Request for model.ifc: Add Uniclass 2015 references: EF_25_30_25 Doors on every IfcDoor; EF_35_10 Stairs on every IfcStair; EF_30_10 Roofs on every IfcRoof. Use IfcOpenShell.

First a look at what the model holds.

```python
import ifcopenshell

model = ifcopenshell.open("model.ifc")
print(model.schema)
print("classifications:", [c.Name for c in model.by_type("IfcClassification")])
for ifc_class in ("IfcDoor", "IfcRoof", "IfcStair", "IfcWall", "IfcWindow"):
    print(ifc_class, len(model.by_type(ifc_class)))
```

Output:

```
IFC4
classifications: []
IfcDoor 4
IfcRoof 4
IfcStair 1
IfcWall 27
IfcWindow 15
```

```python
import ifcopenshell
import ifcopenshell.api.classification

model = ifcopenshell.open("model.ifc")

system = ifcopenshell.api.classification.add_classification(model, classification="Uniclass 2015")

codes = {
    "IfcDoor": ("EF_25_30_25", "Doors"),
    "IfcStair": ("EF_35_10", "Stairs"),
    "IfcRoof": ("EF_30_10", "Roofs"),
}
for ifc_class, (code, name) in codes.items():
    products = model.by_type(ifc_class)
    ifcopenshell.api.classification.add_reference(
        model, products=products, classification=system, identification=code, name=name
    )
    print(code, len(products))

model.write("model_v2.ifc")
```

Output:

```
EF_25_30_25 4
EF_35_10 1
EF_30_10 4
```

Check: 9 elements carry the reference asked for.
